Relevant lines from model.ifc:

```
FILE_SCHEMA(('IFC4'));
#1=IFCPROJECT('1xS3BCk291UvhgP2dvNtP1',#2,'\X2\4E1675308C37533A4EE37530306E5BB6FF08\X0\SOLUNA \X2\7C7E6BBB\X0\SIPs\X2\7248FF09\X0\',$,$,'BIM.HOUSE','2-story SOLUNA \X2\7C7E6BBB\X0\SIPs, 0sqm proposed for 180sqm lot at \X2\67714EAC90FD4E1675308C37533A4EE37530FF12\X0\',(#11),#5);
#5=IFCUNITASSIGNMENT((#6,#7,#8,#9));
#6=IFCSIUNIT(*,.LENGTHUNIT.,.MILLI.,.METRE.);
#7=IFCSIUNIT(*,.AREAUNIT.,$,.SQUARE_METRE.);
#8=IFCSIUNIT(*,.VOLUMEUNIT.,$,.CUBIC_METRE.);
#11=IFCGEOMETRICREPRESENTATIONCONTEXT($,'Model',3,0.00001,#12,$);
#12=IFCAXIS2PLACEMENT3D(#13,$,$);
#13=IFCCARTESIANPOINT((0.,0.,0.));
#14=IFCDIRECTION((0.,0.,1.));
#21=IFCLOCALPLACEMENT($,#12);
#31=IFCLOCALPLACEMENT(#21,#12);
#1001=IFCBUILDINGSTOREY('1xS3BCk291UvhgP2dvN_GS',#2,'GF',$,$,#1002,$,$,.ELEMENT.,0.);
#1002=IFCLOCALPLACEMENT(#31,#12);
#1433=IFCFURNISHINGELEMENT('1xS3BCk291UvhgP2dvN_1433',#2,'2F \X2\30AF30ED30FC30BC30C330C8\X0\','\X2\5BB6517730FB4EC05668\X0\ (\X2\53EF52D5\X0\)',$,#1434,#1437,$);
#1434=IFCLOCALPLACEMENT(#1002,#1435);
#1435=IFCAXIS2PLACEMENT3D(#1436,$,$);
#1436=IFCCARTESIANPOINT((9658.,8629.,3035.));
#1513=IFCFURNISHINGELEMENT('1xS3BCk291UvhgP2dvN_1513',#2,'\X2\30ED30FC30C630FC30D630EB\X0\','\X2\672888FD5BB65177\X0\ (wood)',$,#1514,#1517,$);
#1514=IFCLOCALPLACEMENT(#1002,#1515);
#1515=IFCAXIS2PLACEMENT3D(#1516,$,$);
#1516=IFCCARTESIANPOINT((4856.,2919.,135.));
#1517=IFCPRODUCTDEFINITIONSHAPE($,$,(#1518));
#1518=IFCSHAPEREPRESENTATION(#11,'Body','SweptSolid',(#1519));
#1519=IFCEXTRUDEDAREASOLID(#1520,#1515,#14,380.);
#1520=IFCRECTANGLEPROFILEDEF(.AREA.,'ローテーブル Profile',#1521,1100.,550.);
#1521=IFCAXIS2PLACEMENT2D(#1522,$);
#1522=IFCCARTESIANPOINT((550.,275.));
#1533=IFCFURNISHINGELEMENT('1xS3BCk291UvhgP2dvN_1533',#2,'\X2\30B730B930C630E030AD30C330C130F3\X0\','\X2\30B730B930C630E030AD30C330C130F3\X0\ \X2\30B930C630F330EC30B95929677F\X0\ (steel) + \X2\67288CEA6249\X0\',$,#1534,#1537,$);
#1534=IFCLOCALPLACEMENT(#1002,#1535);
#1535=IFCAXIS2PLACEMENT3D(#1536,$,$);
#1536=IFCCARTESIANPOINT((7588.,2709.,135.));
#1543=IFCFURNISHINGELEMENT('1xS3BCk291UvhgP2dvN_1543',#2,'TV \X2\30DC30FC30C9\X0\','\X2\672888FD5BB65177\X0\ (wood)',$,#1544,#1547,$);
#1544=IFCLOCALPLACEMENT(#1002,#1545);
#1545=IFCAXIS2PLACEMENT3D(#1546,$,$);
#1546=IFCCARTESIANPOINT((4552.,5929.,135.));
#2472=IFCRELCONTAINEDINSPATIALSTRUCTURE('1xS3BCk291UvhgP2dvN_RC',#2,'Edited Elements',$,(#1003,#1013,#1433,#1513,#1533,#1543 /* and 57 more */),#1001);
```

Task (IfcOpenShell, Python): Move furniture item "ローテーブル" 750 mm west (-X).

```python
import ifcopenshell
import ifcopenshell.api.geometry
import ifcopenshell.util.placement
import ifcopenshell.util.unit

model = ifcopenshell.open("model.ifc")
unit_scale = ifcopenshell.util.unit.calculate_unit_scale(model)

item = model.by_id(1513)
matrix = ifcopenshell.util.placement.get_local_placement(item.ObjectPlacement)
matrix[0, 3] -= 0.75 / unit_scale
ifcopenshell.api.geometry.edit_object_placement(model, product=item, matrix=matrix, is_si=False)

print(ifcopenshell.util.placement.get_local_placement(item.ObjectPlacement).round(3) + 0.0)

model.write("model_v2.ifc")
```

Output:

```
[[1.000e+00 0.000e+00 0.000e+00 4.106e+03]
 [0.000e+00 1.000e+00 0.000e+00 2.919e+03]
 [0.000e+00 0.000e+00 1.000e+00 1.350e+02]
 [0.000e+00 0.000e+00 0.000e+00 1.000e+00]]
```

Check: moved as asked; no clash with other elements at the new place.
